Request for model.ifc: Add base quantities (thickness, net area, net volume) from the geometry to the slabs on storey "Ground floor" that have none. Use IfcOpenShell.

First a look at what the model holds.

```python
import ifcopenshell
import ifcopenshell.util.element
import ifcopenshell.util.unit

model = ifcopenshell.open("model.ifc")
print(model.schema)
for unit_type in ("LENGTHUNIT", "AREAUNIT", "VOLUMEUNIT"):
    print(unit_type, ifcopenshell.util.unit.calculate_unit_scale(model, unit_type))
storey = next(s for s in model.by_type("IfcBuildingStorey") if s.Name == "Ground floor")
slabs = [e for e in ifcopenshell.util.element.get_decomposition(storey) if e.is_a("IfcSlab")]
for e in sorted(slabs, key=lambda e: e.id()):
    print(e.id(), e.is_a(), e.Name, list(ifcopenshell.util.element.get_psets(e, qtos_only=True)), sep=" | ")
```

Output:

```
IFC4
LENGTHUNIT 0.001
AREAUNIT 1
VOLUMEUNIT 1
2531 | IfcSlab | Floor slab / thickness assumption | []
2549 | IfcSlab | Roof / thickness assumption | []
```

```python
import ifcopenshell
import ifcopenshell.api.pset
import ifcopenshell.geom
import ifcopenshell.util.element
import ifcopenshell.util.shape
import ifcopenshell.util.unit

model = ifcopenshell.open("model.ifc")
unit_scale = ifcopenshell.util.unit.calculate_unit_scale(model)
area_scale = ifcopenshell.util.unit.calculate_unit_scale(model, "AREAUNIT")
volume_scale = ifcopenshell.util.unit.calculate_unit_scale(model, "VOLUMEUNIT")
settings = ifcopenshell.geom.settings()

storey = next(s for s in model.by_type("IfcBuildingStorey") if s.Name == "Ground floor")
slabs = [e for e in ifcopenshell.util.element.get_decomposition(storey) if e.is_a("IfcSlab")]

for e in sorted(slabs, key=lambda e: e.id()):
    if ifcopenshell.util.element.get_psets(e, qtos_only=True, should_inherit=False):
        continue
    # Geometry comes back in metres, in the element's own axes.
    shape = ifcopenshell.geom.create_shape(settings, e)
    values = {
        "Width": ifcopenshell.util.shape.get_z(shape.geometry) / unit_scale,
        "NetArea": ifcopenshell.util.shape.get_footprint_area(shape.geometry) / area_scale,
        "NetVolume": ifcopenshell.util.shape.get_volume(shape.geometry) / volume_scale,
    }
    qto = ifcopenshell.api.pset.add_qto(model, product=e, name="Qto_SlabBaseQuantities")
    ifcopenshell.api.pset.edit_qto(model, qto=qto, properties=values)
    print(e.id(), {k: round(v, 3) for k, v in values.items()})

model.write("model_v2.ifc")
```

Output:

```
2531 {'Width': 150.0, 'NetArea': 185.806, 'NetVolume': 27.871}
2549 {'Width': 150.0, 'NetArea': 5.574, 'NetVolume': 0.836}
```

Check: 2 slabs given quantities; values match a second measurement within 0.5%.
